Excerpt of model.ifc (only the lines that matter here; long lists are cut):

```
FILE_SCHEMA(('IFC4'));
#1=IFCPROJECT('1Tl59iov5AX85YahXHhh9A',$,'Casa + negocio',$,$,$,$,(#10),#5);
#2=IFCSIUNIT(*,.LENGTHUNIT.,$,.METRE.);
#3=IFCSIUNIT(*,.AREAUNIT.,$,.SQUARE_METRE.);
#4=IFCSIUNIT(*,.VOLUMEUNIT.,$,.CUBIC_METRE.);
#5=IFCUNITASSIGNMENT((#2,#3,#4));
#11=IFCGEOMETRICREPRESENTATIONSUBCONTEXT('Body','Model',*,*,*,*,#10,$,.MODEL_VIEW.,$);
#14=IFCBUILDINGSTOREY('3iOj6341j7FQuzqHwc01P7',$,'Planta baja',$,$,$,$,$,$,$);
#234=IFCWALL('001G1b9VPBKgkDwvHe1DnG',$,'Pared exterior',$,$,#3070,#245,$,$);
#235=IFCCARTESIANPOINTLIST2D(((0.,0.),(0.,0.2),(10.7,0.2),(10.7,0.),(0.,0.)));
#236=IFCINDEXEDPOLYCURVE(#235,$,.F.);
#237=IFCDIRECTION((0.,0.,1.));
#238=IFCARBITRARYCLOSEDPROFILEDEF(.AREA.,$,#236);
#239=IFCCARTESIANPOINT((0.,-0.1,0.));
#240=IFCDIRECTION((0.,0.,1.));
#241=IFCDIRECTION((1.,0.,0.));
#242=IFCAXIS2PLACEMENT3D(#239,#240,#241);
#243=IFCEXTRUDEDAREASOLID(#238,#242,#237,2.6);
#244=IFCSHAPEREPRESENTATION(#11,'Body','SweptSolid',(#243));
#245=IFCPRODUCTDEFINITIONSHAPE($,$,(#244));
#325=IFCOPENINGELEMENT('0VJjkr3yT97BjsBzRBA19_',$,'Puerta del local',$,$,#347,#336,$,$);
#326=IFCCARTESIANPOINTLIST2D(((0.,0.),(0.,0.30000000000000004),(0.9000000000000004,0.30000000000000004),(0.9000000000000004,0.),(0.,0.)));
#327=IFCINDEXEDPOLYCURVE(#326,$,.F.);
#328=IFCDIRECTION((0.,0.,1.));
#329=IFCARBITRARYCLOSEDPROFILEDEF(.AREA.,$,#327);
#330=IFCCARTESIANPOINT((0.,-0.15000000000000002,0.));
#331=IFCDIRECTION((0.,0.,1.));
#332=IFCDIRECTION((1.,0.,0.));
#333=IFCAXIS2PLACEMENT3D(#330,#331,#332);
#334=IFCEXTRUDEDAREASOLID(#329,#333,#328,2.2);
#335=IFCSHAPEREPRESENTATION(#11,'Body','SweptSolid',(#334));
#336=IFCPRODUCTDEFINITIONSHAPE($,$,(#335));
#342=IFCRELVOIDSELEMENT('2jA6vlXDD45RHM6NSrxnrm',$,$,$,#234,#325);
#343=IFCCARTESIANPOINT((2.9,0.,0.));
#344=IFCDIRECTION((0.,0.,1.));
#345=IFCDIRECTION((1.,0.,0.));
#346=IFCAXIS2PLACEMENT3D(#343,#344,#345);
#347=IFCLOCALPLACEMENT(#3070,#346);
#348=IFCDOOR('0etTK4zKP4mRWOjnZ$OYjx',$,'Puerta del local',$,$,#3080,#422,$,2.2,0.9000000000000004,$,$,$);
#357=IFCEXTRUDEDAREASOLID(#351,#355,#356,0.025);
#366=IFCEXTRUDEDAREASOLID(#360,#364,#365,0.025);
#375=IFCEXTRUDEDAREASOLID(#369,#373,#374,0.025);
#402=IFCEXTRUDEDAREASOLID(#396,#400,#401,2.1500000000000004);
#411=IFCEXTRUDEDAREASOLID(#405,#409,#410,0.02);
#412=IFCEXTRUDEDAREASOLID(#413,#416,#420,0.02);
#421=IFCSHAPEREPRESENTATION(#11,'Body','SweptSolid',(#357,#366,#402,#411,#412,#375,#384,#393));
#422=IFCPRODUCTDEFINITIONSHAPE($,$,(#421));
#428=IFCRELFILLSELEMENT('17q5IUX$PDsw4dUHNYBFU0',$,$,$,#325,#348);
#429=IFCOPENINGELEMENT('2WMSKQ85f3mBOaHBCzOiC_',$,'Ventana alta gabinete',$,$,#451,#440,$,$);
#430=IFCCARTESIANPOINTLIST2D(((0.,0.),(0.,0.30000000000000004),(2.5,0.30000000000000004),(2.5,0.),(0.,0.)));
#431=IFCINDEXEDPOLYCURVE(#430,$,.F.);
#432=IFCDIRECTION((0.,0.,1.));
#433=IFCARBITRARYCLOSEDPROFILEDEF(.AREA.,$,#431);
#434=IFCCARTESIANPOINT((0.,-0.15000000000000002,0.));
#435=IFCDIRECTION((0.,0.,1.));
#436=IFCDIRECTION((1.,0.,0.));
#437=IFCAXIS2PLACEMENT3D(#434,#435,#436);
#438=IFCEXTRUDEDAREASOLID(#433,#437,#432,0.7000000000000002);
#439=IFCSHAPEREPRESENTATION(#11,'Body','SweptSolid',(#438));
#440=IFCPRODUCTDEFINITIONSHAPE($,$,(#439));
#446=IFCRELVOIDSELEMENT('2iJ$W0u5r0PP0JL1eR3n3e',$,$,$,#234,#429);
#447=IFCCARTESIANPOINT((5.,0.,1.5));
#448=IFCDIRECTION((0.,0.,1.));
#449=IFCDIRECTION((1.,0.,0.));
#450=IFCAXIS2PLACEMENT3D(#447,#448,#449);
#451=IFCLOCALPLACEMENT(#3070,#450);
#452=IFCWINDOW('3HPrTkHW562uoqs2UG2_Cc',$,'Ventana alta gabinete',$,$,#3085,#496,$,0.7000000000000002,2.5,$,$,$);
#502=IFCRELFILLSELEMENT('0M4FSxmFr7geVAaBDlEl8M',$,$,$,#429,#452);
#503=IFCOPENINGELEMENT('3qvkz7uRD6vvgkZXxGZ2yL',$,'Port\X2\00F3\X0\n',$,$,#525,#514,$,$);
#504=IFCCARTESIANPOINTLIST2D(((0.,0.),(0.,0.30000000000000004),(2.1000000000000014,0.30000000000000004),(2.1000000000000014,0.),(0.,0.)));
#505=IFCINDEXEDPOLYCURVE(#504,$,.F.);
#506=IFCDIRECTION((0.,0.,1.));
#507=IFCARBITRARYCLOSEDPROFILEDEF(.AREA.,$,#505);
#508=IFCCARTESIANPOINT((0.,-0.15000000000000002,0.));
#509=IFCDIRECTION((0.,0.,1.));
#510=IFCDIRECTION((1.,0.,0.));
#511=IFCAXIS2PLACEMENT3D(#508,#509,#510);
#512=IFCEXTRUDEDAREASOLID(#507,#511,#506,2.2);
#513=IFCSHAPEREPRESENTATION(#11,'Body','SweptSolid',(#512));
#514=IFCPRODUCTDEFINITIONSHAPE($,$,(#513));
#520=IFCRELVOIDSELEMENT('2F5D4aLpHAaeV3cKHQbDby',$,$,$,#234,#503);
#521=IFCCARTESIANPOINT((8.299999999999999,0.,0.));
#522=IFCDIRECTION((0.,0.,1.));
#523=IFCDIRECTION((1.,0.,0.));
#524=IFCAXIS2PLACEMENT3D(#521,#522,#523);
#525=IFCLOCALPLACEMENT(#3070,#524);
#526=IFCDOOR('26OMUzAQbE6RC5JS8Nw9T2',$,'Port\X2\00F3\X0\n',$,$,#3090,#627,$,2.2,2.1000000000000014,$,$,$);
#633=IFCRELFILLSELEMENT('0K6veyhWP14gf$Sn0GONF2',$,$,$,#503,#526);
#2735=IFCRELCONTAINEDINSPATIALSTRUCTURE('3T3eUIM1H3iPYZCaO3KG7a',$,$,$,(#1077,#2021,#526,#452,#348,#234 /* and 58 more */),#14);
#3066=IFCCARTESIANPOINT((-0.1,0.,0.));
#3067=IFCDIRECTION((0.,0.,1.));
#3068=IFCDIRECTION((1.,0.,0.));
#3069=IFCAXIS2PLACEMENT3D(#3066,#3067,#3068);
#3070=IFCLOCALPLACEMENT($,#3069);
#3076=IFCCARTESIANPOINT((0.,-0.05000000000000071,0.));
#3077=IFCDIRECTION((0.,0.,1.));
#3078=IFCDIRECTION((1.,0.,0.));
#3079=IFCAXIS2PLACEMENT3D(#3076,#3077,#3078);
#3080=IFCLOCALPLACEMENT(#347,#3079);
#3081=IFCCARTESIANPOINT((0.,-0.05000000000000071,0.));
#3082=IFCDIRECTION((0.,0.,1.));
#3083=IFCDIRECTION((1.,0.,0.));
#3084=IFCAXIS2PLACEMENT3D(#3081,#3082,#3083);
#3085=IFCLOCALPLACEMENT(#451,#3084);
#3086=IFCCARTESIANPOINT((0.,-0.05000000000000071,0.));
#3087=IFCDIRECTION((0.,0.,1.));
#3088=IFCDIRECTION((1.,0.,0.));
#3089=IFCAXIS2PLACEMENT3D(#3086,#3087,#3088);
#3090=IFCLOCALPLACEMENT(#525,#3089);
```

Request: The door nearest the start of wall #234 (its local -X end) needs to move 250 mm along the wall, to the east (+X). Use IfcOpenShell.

```python
import ifcopenshell
import ifcopenshell.api.geometry
import ifcopenshell.util.placement
import ifcopenshell.util.unit

model = ifcopenshell.open("model.ifc")
unit_scale = ifcopenshell.util.unit.calculate_unit_scale(model)

door = model.by_id(348)
opening = door.FillsVoids[0].RelatingOpeningElement
wall = opening.VoidsElements[0].RelatingBuildingElement

wall_matrix = ifcopenshell.util.placement.get_local_placement(wall.ObjectPlacement)
shift = wall_matrix[:3, 0] * 0.25 / unit_scale
before = ifcopenshell.util.placement.get_local_placement(door.ObjectPlacement)[:3, 3].copy()

# The door is placed relative to its opening, so it follows when the opening moves.
matrix = ifcopenshell.util.placement.get_local_placement(opening.ObjectPlacement)
matrix[:3, 3] += shift
ifcopenshell.api.geometry.edit_object_placement(
    model, product=opening, matrix=matrix, is_si=False, should_transform_children=True
)

after = ifcopenshell.util.placement.get_local_placement(door.ObjectPlacement)[:3, 3]
print("door moved by", (after - before).round(3) + 0.0)

model.write("model_v2.ifc")
```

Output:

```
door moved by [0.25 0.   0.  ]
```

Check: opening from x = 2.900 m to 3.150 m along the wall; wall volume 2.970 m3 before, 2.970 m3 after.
